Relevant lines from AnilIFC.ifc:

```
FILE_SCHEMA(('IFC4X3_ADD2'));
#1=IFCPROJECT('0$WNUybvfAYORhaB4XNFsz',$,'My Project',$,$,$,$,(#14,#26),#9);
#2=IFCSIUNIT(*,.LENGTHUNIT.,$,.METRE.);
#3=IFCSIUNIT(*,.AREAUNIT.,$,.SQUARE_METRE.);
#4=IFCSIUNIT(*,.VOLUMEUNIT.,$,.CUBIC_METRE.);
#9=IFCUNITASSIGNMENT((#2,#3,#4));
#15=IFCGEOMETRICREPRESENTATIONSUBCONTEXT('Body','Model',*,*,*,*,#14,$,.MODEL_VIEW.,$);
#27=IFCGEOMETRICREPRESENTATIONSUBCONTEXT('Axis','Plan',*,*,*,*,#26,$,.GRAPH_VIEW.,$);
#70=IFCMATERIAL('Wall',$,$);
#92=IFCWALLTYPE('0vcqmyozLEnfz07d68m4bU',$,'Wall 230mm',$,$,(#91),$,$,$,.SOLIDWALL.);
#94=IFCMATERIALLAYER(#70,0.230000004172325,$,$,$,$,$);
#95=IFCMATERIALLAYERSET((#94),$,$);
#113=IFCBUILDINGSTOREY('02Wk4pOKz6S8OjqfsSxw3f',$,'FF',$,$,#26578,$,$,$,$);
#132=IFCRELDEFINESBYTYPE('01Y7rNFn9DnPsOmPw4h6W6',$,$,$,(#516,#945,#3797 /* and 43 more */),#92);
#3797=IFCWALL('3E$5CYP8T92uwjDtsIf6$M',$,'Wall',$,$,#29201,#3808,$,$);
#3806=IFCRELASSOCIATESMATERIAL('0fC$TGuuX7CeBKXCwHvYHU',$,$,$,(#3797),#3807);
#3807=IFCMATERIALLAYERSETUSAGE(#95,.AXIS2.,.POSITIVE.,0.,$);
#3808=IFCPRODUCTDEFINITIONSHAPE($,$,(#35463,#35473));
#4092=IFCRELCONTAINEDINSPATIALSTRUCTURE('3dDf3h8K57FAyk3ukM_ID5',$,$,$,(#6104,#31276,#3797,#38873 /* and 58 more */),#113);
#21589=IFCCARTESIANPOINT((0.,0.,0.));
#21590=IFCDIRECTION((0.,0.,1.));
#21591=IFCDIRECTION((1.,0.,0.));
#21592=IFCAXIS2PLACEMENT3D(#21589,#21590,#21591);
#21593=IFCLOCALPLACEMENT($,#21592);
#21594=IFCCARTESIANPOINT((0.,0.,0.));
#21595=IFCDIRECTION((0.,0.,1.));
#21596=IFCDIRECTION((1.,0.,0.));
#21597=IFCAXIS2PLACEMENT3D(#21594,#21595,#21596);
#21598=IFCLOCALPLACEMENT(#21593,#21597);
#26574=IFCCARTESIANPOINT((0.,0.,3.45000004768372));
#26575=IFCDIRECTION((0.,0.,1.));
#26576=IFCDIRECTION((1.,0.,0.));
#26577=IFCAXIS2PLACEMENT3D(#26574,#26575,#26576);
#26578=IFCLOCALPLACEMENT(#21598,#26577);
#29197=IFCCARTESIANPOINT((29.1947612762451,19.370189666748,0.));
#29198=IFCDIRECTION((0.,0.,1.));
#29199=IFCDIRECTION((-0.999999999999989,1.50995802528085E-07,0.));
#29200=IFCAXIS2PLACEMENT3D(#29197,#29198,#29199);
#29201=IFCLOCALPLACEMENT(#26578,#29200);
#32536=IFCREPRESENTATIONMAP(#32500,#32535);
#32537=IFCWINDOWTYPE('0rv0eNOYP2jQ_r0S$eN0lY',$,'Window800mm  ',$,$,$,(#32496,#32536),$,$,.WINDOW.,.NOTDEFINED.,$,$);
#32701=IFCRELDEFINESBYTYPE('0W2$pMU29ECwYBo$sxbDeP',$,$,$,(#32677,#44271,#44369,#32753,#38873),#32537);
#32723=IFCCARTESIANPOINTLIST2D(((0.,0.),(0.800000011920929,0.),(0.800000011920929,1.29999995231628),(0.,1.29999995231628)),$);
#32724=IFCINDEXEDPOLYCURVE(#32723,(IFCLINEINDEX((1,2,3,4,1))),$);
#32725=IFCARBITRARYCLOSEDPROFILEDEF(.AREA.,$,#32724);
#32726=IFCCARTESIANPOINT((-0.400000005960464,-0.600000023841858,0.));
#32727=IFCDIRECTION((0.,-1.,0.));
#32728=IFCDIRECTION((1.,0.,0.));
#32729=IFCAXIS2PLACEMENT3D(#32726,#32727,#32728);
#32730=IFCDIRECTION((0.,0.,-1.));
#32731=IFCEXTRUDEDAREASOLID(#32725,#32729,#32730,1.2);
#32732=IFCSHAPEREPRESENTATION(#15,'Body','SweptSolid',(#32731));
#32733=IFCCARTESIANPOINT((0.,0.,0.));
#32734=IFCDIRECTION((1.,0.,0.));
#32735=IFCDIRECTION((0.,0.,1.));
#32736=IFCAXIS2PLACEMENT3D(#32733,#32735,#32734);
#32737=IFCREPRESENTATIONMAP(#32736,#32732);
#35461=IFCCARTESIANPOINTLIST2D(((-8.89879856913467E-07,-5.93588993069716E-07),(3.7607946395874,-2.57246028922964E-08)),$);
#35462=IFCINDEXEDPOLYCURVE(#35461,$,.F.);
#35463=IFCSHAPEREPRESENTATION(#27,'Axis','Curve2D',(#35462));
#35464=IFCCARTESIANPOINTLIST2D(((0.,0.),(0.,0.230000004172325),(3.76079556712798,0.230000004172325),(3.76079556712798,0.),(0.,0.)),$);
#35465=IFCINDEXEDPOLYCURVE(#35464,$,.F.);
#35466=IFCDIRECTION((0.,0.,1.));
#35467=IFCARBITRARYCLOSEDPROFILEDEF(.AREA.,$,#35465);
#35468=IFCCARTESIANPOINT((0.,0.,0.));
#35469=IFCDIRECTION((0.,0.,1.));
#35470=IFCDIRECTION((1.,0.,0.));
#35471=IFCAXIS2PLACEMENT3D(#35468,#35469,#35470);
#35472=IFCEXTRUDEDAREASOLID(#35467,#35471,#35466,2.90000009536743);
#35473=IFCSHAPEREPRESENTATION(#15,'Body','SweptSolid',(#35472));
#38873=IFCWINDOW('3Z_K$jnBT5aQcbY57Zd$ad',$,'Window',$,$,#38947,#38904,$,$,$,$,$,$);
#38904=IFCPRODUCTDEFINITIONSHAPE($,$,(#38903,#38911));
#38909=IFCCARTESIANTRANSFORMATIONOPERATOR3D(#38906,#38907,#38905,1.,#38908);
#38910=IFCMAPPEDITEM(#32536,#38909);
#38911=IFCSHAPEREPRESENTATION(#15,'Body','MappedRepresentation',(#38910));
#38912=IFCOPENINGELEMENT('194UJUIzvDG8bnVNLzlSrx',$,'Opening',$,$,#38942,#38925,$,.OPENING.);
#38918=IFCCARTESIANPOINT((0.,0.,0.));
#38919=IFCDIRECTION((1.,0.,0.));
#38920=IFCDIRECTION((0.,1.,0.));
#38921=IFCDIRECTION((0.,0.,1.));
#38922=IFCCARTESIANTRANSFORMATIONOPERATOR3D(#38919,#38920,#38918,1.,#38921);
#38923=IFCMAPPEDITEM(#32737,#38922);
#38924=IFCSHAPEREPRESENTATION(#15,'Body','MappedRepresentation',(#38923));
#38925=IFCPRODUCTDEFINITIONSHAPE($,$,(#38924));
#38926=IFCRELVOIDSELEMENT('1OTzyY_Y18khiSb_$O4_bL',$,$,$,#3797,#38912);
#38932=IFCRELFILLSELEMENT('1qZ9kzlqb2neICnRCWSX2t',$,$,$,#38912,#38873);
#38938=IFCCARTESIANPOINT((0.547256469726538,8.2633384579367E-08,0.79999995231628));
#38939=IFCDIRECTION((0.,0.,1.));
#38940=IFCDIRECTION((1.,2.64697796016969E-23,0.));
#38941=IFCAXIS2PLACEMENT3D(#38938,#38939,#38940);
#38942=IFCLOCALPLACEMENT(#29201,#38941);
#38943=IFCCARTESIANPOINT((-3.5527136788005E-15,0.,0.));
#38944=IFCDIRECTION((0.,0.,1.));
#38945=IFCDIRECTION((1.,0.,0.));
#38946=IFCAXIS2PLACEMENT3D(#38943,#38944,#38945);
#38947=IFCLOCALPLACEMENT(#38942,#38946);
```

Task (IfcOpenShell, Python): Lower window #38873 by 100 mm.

```python
import numpy as np
import ifcopenshell
import ifcopenshell.api.geometry
import ifcopenshell.util.placement
import ifcopenshell.util.unit

model = ifcopenshell.open("AnilIFC.ifc")
unit_scale = ifcopenshell.util.unit.calculate_unit_scale(model)

window = model.by_guid("3Z_K$jnBT5aQcbY57Zd$ad")
opening = window.FillsVoids[0].RelatingOpeningElement
dz = -0.1

shift = np.array([0.0, 0.0, dz])
# The window is placed relative to its opening, so it follows when the opening moves.
matrix = ifcopenshell.util.placement.get_local_placement(opening.ObjectPlacement)
matrix[:3, 3] += shift
ifcopenshell.api.geometry.edit_object_placement(
    model, product=opening, matrix=matrix, is_si=False, should_transform_children=True
)

print(f"moved by {dz * unit_scale:+.3f} m")

model.write("AnilIFC-out.ifc")
```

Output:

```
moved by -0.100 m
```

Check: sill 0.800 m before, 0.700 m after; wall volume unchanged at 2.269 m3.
